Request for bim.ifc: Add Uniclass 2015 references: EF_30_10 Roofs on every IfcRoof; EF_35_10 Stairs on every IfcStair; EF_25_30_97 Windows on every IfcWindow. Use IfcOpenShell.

First a look at what the model holds.

```python
import ifcopenshell

model = ifcopenshell.open("bim.ifc")
print(model.schema)
print("classifications:", [c.Name for c in model.by_type("IfcClassification")])
for ifc_class in ("IfcDoor", "IfcRoof", "IfcStair", "IfcWall", "IfcWindow"):
    print(ifc_class, len(model.by_type(ifc_class)))
```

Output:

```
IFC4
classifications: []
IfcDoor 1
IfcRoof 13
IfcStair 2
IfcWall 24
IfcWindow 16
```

```python
import ifcopenshell
import ifcopenshell.api.classification

model = ifcopenshell.open("bim.ifc")

system = ifcopenshell.api.classification.add_classification(model, classification="Uniclass 2015")

codes = {
    "IfcRoof": ("EF_30_10", "Roofs"),
    "IfcStair": ("EF_35_10", "Stairs"),
    "IfcWindow": ("EF_25_30_97", "Windows"),
}
for ifc_class, (code, name) in codes.items():
    products = model.by_type(ifc_class)
    ifcopenshell.api.classification.add_reference(
        model, products=products, classification=system, identification=code, name=name
    )
    print(code, len(products))

model.write("bim-out.ifc")
```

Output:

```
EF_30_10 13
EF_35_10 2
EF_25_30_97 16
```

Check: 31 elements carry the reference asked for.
